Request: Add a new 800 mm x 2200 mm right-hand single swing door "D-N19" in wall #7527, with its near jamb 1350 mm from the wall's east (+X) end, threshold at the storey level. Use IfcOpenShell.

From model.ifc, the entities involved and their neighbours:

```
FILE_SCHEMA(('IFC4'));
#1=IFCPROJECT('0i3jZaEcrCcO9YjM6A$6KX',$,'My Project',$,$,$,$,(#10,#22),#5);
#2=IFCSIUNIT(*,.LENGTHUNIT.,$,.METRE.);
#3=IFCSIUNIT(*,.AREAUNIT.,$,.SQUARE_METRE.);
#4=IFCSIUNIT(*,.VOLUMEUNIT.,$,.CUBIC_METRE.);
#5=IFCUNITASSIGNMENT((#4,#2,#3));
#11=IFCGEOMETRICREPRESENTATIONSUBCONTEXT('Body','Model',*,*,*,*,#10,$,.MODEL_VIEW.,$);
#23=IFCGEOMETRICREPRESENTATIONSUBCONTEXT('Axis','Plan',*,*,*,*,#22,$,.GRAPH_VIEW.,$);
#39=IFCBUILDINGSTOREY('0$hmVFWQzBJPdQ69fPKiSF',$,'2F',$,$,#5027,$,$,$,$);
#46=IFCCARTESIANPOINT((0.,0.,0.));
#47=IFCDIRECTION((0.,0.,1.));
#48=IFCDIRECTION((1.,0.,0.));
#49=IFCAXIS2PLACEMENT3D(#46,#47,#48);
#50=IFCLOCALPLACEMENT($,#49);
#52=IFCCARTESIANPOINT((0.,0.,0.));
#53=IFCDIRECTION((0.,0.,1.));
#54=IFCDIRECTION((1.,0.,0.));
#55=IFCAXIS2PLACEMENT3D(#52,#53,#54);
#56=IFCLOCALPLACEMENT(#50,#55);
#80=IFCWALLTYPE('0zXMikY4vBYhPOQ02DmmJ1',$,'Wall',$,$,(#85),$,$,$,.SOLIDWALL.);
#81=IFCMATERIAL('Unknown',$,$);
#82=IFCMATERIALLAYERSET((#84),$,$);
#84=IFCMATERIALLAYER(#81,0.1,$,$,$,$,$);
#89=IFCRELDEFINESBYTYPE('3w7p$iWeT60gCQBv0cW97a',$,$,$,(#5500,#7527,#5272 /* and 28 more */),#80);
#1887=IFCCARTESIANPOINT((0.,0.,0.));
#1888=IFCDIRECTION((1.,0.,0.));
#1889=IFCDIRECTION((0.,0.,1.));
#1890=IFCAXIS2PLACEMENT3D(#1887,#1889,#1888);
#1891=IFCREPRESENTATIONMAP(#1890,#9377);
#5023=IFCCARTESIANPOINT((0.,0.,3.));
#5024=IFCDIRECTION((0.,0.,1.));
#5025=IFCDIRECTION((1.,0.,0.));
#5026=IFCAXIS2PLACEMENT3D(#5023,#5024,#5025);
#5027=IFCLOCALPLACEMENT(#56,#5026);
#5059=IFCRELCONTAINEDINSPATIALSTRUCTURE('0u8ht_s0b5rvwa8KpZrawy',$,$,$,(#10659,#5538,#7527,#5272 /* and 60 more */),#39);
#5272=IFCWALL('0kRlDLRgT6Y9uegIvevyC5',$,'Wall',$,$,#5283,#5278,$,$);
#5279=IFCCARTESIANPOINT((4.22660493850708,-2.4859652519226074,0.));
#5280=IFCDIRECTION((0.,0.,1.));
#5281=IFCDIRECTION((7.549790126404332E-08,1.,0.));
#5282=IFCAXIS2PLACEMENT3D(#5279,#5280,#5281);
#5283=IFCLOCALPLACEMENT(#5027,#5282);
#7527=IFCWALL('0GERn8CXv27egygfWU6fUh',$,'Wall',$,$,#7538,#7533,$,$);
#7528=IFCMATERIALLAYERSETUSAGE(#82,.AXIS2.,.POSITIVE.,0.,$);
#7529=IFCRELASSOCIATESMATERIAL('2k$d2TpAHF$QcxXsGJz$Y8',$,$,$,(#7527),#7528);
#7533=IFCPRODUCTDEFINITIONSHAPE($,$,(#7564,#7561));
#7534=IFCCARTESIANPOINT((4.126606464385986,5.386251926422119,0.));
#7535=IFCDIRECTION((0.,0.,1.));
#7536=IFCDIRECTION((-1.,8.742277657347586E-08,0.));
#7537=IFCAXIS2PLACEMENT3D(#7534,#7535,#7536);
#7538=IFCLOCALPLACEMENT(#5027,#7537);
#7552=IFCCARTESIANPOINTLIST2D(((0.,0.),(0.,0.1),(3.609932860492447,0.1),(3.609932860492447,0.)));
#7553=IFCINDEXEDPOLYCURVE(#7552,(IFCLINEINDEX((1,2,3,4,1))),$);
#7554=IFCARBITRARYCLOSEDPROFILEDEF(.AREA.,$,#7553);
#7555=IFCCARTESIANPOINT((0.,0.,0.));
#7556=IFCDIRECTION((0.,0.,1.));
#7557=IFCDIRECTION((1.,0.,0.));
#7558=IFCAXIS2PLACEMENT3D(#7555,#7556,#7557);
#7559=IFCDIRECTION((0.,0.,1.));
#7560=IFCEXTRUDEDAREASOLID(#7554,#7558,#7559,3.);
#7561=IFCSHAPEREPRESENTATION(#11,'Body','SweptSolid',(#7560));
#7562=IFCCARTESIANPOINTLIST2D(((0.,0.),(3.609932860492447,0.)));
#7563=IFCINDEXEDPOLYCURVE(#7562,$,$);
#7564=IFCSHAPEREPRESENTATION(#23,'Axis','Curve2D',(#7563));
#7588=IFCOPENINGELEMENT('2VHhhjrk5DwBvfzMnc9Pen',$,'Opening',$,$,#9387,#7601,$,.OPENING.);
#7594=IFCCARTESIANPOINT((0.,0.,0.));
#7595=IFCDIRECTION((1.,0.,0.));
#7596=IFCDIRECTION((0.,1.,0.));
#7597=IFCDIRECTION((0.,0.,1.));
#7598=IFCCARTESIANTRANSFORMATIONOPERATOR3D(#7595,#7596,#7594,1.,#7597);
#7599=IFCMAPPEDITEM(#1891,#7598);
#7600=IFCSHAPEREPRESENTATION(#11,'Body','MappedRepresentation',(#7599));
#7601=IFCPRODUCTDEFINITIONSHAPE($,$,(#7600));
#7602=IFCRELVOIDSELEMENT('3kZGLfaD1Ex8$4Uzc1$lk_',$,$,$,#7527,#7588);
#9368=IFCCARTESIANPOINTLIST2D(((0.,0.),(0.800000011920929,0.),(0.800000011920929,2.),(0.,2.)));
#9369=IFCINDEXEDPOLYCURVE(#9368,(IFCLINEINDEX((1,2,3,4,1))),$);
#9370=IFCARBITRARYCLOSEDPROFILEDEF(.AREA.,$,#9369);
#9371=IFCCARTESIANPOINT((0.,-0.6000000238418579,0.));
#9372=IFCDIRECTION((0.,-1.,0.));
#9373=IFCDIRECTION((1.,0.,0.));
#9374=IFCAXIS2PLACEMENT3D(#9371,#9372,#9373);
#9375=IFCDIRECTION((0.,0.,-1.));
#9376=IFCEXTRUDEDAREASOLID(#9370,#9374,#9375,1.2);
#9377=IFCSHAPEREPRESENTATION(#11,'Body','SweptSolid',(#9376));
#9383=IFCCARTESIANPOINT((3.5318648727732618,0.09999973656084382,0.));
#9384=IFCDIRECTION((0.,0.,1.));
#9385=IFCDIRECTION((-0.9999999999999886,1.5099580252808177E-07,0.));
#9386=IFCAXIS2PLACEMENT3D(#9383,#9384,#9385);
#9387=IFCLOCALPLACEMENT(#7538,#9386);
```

```python
import numpy as np
import ifcopenshell
import ifcopenshell.api.feature
import ifcopenshell.api.geometry
import ifcopenshell.api.root
import ifcopenshell.api.spatial
import ifcopenshell.geom
import ifcopenshell.util.element
import ifcopenshell.util.placement
import ifcopenshell.util.representation
import ifcopenshell.util.shape
import ifcopenshell.util.unit

model = ifcopenshell.open("model.ifc")
unit_scale = ifcopenshell.util.unit.calculate_unit_scale(model)
settings = ifcopenshell.geom.settings()


def volume(element):
    """Net volume in cubic metres, openings subtracted."""
    shape = ifcopenshell.geom.create_shape(settings, element)
    return ifcopenshell.util.shape.get_volume(shape.geometry)


wall = model.by_id(7527)
storey = ifcopenshell.util.element.get_container(wall, ifc_class="IfcBuildingStorey")
context = ifcopenshell.util.representation.get_context(model, "Model", "Body", "MODEL_VIEW")
before = volume(wall)

width, height, from_end, sill = 0.8, 2.2, 1.35, 0.0  # metres

# The wall runs along its own X axis, and the end named is its -X end.
wall_shape = ifcopenshell.geom.create_shape(settings, wall)
x, y, z = ifcopenshell.util.shape.get_vertices(wall_shape.geometry).T
start = x.min() + from_end
face, thickness = float(y.min()), float(y.max() - y.min())
wall_matrix = ifcopenshell.util.placement.get_local_placement(wall.ObjectPlacement)
level = ifcopenshell.util.placement.get_local_placement(storey.ObjectPlacement)[2, 3]


def in_wall(x, y):
    """Placement at x, y metres in the wall's axes, at sill height."""
    matrix = wall_matrix.copy()
    matrix[:, 3] = wall_matrix @ np.array([x / unit_scale, y / unit_scale, 0.0, 1.0])
    matrix[2, 3] = level + sill / unit_scale
    return matrix


# Opening: a box that overshoots both wall faces by 50 mm.
opening = ifcopenshell.api.root.create_entity(model, ifc_class="IfcOpeningElement", predefined_type="OPENING")
box = ifcopenshell.api.geometry.add_wall_representation(
    model, context=context, length=width, height=height, thickness=thickness + 0.1
)
ifcopenshell.api.geometry.assign_representation(model, product=opening, representation=box)
ifcopenshell.api.geometry.edit_object_placement(model, product=opening, matrix=in_wall(start, face - 0.05), is_si=False)
ifcopenshell.api.feature.add_feature(model, feature=opening, element=wall)

door = ifcopenshell.api.root.create_entity(model, ifc_class="IfcDoor", name="D-N19", predefined_type="DOOR")
door.OverallWidth, door.OverallHeight = width / unit_scale, height / unit_scale
door.OperationType = "SINGLE_SWING_RIGHT"
body = ifcopenshell.api.geometry.add_door_representation(
    model,
    context=context,
    overall_width=door.OverallWidth,
    overall_height=door.OverallHeight,
    operation_type="SINGLE_SWING_RIGHT",
    lining_properties={"LiningDepth": thickness / unit_scale, "ThresholdDepth": thickness / unit_scale},
)
ifcopenshell.api.geometry.assign_representation(model, product=door, representation=body)
ifcopenshell.api.spatial.assign_container(model, products=[door], relating_structure=storey)
ifcopenshell.api.feature.add_filling(model, opening=opening, element=door)

# The lining spans the wall, so the door starts at the wall face.
ifcopenshell.api.geometry.edit_object_placement(model, product=door, matrix=in_wall(start, face), is_si=False)

after = volume(wall)

print(f"wall volume {before:.3f} -> {after:.3f} m3")

model.write("model_updated.ifc")
```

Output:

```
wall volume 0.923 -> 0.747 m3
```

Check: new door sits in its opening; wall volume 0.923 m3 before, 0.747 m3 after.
